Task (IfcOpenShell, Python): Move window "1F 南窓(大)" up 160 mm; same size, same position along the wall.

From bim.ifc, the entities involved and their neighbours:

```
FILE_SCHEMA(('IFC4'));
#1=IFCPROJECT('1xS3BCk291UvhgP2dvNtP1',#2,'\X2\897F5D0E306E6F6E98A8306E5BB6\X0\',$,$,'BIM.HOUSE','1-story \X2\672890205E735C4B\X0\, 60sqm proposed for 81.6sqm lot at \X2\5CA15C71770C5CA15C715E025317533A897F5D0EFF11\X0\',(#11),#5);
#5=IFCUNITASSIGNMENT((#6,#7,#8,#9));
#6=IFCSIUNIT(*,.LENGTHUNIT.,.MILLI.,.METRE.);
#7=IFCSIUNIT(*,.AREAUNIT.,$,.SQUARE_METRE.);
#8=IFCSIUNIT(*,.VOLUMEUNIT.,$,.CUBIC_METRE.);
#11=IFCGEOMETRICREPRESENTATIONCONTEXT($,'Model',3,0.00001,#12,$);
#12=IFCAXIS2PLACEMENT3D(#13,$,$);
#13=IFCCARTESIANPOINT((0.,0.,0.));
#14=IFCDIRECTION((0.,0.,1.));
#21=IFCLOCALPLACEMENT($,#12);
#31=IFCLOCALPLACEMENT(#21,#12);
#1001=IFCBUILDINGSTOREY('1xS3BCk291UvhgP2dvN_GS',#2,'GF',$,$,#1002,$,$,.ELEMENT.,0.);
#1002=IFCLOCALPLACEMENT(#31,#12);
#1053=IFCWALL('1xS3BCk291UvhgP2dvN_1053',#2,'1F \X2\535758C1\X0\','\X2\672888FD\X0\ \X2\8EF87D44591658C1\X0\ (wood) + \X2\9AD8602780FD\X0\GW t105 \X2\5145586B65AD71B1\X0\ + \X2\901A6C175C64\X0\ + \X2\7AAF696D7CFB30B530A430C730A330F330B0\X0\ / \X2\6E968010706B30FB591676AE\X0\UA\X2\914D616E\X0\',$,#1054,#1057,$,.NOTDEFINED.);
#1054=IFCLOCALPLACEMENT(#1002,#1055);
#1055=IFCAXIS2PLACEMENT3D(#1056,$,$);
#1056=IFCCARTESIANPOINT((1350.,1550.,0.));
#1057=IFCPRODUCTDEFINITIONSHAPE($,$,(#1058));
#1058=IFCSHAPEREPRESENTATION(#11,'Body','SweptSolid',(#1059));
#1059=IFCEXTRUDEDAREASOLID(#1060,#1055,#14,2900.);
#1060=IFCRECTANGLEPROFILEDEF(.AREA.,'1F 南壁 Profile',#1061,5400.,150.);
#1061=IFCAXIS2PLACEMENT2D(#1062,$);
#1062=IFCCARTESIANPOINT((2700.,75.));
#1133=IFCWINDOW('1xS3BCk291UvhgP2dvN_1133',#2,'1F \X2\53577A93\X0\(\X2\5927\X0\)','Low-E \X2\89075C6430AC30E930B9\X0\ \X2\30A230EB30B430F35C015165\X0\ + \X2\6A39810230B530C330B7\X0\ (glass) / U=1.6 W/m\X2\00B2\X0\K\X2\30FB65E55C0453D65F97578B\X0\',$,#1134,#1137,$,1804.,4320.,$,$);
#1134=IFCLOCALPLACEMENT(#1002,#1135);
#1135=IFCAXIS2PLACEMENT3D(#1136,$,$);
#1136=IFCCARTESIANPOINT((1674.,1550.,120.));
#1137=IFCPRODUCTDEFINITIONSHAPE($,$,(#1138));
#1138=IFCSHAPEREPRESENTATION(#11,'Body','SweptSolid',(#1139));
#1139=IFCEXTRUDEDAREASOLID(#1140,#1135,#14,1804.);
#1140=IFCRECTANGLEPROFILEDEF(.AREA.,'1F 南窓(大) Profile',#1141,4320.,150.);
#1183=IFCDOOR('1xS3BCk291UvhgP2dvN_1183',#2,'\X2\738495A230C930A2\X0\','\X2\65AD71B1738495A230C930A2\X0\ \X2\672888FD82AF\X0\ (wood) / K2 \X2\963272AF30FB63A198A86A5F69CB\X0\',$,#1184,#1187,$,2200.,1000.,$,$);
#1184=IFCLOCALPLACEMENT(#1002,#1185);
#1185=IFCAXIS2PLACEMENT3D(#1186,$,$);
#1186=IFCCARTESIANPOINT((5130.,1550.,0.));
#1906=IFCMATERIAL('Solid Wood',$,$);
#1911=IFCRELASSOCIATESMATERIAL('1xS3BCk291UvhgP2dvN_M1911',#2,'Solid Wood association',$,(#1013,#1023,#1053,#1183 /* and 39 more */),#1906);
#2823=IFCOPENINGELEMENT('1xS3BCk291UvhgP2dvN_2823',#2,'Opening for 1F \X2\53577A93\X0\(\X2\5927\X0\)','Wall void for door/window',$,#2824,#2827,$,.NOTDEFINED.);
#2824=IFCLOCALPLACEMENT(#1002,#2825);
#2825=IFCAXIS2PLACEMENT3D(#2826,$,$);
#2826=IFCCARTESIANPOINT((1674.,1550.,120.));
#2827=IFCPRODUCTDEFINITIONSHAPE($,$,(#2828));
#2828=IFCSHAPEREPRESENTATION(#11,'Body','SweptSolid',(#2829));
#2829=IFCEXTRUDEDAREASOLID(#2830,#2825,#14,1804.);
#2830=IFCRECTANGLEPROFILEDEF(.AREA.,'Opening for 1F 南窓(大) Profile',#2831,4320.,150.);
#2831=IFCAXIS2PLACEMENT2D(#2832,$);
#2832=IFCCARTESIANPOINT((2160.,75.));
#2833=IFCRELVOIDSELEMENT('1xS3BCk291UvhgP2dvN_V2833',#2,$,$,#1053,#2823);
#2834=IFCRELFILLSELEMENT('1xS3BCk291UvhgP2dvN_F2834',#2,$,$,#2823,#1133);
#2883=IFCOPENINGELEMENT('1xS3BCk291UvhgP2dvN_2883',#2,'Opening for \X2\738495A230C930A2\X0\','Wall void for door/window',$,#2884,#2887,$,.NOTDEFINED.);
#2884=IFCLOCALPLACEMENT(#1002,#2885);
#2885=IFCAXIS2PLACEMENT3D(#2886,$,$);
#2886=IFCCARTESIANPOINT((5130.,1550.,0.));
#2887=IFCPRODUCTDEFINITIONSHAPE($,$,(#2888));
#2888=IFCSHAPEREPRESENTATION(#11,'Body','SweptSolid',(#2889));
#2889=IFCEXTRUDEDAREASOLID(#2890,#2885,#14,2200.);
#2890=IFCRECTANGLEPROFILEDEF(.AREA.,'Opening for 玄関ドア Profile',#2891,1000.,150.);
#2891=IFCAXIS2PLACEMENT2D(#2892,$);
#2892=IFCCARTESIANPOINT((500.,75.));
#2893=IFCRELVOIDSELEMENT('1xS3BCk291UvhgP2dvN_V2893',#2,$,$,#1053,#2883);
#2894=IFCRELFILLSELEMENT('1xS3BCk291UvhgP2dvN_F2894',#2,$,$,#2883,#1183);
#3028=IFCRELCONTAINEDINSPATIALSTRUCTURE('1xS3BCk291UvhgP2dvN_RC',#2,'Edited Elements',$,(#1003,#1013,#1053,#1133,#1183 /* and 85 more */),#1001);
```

```python
import numpy as np
import ifcopenshell
import ifcopenshell.api.geometry
import ifcopenshell.util.placement
import ifcopenshell.util.unit

model = ifcopenshell.open("bim.ifc")
unit_scale = ifcopenshell.util.unit.calculate_unit_scale(model)

window = model.by_id(1133)
opening = window.FillsVoids[0].RelatingOpeningElement
dz = 0.16 / unit_scale

shift = np.array([0.0, 0.0, dz])
# The window is not placed relative to its opening, so move both.
for product in (opening, window):
    matrix = ifcopenshell.util.placement.get_local_placement(product.ObjectPlacement)
    matrix[:3, 3] += shift
    ifcopenshell.api.geometry.edit_object_placement(model, product=product, matrix=matrix, is_si=False)

print(f"moved by {dz * unit_scale:+.3f} m")

model.write("bim_updated.ifc")
```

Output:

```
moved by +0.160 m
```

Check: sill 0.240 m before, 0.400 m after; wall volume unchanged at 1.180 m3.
